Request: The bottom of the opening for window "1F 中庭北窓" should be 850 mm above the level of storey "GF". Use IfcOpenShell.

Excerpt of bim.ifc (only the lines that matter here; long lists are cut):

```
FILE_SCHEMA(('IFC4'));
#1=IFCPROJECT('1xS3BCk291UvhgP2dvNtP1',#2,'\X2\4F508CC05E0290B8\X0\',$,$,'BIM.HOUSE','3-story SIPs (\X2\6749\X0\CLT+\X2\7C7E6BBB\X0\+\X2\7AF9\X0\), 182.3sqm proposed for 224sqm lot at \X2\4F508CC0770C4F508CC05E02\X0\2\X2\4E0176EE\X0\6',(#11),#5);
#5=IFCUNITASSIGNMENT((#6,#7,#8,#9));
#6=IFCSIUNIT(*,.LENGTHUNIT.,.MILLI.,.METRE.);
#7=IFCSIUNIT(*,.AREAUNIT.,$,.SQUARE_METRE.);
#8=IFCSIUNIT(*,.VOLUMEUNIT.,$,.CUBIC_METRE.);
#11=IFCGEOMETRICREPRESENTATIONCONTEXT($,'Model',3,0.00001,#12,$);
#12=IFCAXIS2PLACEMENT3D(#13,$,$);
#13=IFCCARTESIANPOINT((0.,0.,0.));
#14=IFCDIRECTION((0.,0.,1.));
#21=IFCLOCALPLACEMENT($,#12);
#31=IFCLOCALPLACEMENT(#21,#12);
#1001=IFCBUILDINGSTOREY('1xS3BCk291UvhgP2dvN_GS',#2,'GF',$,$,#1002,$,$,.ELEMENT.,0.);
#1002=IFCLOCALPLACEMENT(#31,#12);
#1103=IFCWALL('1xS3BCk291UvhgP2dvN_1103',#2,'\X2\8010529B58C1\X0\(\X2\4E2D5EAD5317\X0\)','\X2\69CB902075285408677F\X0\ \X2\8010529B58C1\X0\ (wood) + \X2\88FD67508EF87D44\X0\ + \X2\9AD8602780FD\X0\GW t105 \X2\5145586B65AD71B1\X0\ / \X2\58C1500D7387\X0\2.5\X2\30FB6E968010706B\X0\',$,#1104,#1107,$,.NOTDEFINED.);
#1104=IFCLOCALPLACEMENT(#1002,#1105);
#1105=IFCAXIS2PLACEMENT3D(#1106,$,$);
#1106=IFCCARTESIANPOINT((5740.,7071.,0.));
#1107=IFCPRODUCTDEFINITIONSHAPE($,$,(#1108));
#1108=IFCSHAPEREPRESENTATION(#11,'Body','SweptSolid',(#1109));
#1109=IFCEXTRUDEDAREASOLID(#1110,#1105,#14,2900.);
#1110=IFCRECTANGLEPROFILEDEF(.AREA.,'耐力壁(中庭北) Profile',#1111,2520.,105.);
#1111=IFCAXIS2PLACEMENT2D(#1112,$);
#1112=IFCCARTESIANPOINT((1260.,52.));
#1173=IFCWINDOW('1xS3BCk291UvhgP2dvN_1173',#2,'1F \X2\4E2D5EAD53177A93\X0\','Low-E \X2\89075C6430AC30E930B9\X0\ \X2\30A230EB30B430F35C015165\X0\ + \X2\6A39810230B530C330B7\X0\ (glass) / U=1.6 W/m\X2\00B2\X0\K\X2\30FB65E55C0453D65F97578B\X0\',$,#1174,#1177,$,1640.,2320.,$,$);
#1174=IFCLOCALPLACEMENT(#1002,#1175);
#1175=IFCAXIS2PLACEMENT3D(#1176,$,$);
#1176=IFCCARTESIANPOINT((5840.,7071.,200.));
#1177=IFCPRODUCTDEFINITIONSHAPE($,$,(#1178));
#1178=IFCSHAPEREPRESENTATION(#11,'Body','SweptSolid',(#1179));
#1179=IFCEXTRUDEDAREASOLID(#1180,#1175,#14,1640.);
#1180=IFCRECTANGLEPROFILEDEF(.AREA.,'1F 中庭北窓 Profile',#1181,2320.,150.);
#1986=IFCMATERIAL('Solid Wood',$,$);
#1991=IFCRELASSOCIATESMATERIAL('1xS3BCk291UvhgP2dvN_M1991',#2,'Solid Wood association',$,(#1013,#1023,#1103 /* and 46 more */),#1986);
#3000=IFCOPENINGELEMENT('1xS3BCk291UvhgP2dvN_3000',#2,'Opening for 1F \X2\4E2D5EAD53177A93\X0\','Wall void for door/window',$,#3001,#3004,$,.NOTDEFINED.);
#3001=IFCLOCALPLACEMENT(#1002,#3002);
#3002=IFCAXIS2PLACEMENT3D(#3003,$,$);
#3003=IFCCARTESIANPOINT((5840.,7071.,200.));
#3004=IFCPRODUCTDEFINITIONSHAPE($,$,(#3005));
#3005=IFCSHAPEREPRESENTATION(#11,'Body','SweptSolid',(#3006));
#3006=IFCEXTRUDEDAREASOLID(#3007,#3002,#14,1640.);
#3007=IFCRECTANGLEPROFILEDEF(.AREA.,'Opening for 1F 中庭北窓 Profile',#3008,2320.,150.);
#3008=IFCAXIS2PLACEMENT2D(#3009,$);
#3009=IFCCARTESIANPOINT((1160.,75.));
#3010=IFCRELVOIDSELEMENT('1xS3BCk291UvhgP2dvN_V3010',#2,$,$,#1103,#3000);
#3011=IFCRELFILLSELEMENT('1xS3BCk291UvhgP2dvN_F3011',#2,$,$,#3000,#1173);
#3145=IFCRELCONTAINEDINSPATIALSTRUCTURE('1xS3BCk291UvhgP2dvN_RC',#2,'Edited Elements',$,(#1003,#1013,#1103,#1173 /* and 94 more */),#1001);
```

```python
import numpy as np
import ifcopenshell
import ifcopenshell.api.geometry
import ifcopenshell.geom
import ifcopenshell.util.element
import ifcopenshell.util.placement
import ifcopenshell.util.shape
import ifcopenshell.util.unit

model = ifcopenshell.open("bim.ifc")
unit_scale = ifcopenshell.util.unit.calculate_unit_scale(model)

window = model.by_guid("1xS3BCk291UvhgP2dvN_1173")
opening = window.FillsVoids[0].RelatingOpeningElement
storey = ifcopenshell.util.element.get_container(window, ifc_class="IfcBuildingStorey")
level = ifcopenshell.util.placement.get_local_placement(storey.ObjectPlacement)[2, 3]

# The opening's origin need not be at the sill, so measure its lowest point.
shape = ifcopenshell.geom.create_shape(ifcopenshell.geom.settings(), opening)
bottom = ifcopenshell.util.shape.get_shape_bottom_elevation(shape, shape.geometry) / unit_scale
dz = level + 0.85 / unit_scale - bottom

shift = np.array([0.0, 0.0, dz])
# The window is not placed relative to its opening, so move both.
for product in (opening, window):
    matrix = ifcopenshell.util.placement.get_local_placement(product.ObjectPlacement)
    matrix[:3, 3] += shift
    ifcopenshell.api.geometry.edit_object_placement(model, product=product, matrix=matrix, is_si=False)

print(f"moved by {dz * unit_scale:+.3f} m")

model.write("bim_v2.ifc")
```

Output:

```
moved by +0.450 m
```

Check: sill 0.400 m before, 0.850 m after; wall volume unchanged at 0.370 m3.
